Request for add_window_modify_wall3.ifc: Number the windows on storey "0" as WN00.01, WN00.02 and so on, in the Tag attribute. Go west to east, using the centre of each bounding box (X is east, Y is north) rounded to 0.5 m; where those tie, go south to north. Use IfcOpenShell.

First a look at what the model holds.

```python
import ifcopenshell
import ifcopenshell.util.element
import ifcopenshell.util.placement

model = ifcopenshell.open("add_window_modify_wall3.ifc")
print(model.schema)
storey = next(s for s in model.by_type("IfcBuildingStorey") if s.Name == "0")
windows = [e for e in ifcopenshell.util.element.get_decomposition(storey) if e.is_a("IfcWindow")]
for e in sorted(windows, key=lambda e: e.id()):
    origin = ifcopenshell.util.placement.get_local_placement(e.ObjectPlacement)[:3, 3]
    print(e.id(), e.Tag, e.Name, origin.round(2) + 0.0, sep=" | ")
```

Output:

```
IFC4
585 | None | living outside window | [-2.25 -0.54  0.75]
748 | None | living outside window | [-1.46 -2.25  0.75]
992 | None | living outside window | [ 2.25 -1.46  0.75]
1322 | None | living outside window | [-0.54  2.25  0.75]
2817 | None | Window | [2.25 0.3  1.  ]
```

```python
import ifcopenshell
import ifcopenshell.geom
import ifcopenshell.util.element
import ifcopenshell.util.shape

model = ifcopenshell.open("add_window_modify_wall3.ifc")
settings = ifcopenshell.geom.settings()
settings.set("use-world-coords", True)


def centre(element):
    shape = ifcopenshell.geom.create_shape(settings, element)
    return ifcopenshell.util.shape.get_bbox_centroid(shape.geometry)


storey = next(s for s in model.by_type("IfcBuildingStorey") if s.Name == "0")
windows = [e for e in ifcopenshell.util.element.get_decomposition(storey) if e.is_a("IfcWindow")]

# Insertion points can sit at a corner or the storey origin, so sort by the geometry (in metres).
centres = {e: centre(e) for e in windows}
windows.sort(key=lambda e: (round(centres[e][0] / 0.5), centres[e][1]))

for i, e in enumerate(windows, start=1):
    number = f"WN00.{i:02d}"
    e.Tag = number
    print(e.id(), number)

model.write("add_window_modify_wall3_edited.ifc")
```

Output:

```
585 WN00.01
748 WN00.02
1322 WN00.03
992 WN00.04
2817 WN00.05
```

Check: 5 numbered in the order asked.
